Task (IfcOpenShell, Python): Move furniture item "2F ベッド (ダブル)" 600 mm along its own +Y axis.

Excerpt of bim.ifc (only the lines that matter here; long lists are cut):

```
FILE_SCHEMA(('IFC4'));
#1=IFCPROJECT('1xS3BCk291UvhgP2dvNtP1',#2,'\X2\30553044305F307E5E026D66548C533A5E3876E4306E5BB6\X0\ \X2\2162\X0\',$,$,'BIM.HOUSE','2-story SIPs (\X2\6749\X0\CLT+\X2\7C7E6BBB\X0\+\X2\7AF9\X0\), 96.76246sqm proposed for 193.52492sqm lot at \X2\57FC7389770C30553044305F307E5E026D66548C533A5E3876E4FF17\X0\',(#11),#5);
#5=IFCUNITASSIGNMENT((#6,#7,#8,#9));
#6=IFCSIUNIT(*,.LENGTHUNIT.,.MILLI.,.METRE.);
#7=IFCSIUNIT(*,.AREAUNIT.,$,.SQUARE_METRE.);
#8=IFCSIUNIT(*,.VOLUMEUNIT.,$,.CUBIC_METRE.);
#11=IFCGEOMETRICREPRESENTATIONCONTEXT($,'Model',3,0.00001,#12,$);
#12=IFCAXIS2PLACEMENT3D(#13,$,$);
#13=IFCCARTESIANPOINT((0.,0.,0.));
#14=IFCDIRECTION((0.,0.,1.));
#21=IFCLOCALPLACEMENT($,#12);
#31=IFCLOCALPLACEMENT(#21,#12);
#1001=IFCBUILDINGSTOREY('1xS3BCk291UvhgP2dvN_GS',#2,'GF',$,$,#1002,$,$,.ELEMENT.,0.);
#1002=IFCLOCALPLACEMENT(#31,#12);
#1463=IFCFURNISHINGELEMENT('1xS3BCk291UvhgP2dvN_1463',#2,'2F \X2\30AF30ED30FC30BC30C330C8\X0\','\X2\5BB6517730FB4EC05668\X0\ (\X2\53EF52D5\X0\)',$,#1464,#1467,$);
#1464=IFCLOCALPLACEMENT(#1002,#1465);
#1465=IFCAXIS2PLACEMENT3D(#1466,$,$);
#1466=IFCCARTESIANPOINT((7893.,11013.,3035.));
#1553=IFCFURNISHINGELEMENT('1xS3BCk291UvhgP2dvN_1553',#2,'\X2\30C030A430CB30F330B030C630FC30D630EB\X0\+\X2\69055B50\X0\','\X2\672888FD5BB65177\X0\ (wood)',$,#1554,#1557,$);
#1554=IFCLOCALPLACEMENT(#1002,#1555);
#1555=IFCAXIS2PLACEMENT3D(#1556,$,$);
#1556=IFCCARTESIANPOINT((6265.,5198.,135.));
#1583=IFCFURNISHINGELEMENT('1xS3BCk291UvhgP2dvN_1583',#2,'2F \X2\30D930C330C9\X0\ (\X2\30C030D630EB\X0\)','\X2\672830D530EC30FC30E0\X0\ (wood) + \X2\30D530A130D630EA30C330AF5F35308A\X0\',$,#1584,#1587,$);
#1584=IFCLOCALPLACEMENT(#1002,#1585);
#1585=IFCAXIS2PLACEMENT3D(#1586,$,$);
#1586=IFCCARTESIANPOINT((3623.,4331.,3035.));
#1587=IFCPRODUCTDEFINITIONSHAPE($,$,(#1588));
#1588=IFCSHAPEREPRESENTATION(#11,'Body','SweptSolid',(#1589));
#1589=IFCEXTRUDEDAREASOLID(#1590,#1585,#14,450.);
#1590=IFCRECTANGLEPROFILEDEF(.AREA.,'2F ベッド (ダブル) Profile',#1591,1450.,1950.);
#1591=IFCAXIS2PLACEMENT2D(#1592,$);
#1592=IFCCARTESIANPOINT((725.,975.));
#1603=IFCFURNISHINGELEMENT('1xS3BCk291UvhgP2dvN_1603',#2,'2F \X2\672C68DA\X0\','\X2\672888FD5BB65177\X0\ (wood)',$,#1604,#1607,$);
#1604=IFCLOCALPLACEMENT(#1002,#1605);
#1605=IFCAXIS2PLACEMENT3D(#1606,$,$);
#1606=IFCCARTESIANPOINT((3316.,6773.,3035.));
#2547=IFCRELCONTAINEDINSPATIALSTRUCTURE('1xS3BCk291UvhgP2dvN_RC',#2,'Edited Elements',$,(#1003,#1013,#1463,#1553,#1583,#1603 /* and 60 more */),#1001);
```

```python
import ifcopenshell
import ifcopenshell.api.geometry
import ifcopenshell.util.placement
import ifcopenshell.util.unit

model = ifcopenshell.open("bim.ifc")
unit_scale = ifcopenshell.util.unit.calculate_unit_scale(model)

item = model.by_guid("1xS3BCk291UvhgP2dvN_1583")
matrix = ifcopenshell.util.placement.get_local_placement(item.ObjectPlacement)
matrix[:3, 3] += matrix[:3, 1] * 0.6 / unit_scale
ifcopenshell.api.geometry.edit_object_placement(model, product=item, matrix=matrix, is_si=False)

print(ifcopenshell.util.placement.get_local_placement(item.ObjectPlacement).round(3) + 0.0)

model.write("bim_rev.ifc")
```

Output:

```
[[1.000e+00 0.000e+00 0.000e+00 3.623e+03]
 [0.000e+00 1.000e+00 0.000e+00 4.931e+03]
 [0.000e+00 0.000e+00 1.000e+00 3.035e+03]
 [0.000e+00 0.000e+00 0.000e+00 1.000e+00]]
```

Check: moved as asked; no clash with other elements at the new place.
